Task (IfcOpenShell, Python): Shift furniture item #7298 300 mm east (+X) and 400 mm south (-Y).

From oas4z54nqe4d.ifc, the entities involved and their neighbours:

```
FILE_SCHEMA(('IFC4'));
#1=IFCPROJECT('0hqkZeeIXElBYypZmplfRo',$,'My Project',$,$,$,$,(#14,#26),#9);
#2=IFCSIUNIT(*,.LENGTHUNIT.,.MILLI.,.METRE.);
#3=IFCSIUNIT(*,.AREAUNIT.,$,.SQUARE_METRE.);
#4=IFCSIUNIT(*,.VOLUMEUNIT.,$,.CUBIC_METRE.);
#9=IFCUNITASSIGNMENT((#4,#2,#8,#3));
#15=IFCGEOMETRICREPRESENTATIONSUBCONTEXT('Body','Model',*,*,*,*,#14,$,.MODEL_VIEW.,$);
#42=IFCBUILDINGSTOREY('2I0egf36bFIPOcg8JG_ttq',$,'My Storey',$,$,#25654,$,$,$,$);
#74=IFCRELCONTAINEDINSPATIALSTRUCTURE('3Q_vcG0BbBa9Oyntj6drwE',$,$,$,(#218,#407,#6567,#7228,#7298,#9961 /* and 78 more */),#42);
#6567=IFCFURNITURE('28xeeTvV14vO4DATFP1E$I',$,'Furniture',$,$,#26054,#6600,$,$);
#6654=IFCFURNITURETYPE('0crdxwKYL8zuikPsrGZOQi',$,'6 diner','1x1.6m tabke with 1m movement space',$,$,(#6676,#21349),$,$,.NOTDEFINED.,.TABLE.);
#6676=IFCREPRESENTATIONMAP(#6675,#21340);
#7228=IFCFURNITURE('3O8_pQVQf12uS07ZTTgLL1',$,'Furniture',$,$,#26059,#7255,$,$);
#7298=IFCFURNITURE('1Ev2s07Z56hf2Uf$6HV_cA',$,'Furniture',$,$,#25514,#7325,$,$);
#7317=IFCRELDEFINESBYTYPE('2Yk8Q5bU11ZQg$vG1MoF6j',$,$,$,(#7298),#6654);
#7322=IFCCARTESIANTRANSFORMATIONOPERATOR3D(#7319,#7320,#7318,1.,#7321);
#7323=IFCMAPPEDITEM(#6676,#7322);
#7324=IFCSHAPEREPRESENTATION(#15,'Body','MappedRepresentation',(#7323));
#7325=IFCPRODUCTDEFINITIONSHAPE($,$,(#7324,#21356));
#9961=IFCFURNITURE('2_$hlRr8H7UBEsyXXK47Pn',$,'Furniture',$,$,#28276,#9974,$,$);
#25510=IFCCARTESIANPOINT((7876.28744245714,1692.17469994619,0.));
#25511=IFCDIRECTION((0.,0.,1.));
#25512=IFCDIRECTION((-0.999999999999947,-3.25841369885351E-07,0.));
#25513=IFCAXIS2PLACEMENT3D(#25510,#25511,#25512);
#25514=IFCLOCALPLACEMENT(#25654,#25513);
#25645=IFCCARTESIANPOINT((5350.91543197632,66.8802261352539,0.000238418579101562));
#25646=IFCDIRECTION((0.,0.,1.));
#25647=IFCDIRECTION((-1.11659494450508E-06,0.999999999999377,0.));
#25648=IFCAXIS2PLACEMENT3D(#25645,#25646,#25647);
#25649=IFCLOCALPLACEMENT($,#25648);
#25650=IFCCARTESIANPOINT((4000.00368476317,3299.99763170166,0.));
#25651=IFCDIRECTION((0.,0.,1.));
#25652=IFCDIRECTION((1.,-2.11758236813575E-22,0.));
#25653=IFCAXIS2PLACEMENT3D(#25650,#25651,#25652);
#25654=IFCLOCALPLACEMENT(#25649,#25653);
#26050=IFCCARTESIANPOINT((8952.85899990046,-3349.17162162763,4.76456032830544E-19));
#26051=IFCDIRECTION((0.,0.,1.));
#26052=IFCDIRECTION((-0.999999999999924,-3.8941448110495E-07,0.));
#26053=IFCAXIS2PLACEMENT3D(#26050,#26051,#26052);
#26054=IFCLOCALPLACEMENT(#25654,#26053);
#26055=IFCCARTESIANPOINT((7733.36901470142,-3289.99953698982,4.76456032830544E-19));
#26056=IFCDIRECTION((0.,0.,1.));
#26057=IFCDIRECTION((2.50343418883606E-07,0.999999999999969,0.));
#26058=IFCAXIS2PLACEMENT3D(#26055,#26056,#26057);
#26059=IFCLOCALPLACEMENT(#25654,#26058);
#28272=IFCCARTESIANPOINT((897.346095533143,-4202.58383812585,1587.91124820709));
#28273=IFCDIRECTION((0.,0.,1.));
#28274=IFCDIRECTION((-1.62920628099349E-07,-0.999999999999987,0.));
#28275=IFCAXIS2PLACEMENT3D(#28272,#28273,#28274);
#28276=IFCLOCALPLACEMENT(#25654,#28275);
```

```python
import ifcopenshell
import ifcopenshell.api.geometry
import ifcopenshell.util.placement

model = ifcopenshell.open("oas4z54nqe4d.ifc")

item = model.by_guid("1Ev2s07Z56hf2Uf$6HV_cA")
matrix = ifcopenshell.util.placement.get_local_placement(item.ObjectPlacement)
matrix[0, 3] += 300.0
matrix[1, 3] -= 400.0
ifcopenshell.api.geometry.edit_object_placement(model, product=item, matrix=matrix, is_si=False)

print(ifcopenshell.util.placement.get_local_placement(item.ObjectPlacement).round(3) + 0.0)

model.write("oas4z54nqe4d_v2.ifc")
```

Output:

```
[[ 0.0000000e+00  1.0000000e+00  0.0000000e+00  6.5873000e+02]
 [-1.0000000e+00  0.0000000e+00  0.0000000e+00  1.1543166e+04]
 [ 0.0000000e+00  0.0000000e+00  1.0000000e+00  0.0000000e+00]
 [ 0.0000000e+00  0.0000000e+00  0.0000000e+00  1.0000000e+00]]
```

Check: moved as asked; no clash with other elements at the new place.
